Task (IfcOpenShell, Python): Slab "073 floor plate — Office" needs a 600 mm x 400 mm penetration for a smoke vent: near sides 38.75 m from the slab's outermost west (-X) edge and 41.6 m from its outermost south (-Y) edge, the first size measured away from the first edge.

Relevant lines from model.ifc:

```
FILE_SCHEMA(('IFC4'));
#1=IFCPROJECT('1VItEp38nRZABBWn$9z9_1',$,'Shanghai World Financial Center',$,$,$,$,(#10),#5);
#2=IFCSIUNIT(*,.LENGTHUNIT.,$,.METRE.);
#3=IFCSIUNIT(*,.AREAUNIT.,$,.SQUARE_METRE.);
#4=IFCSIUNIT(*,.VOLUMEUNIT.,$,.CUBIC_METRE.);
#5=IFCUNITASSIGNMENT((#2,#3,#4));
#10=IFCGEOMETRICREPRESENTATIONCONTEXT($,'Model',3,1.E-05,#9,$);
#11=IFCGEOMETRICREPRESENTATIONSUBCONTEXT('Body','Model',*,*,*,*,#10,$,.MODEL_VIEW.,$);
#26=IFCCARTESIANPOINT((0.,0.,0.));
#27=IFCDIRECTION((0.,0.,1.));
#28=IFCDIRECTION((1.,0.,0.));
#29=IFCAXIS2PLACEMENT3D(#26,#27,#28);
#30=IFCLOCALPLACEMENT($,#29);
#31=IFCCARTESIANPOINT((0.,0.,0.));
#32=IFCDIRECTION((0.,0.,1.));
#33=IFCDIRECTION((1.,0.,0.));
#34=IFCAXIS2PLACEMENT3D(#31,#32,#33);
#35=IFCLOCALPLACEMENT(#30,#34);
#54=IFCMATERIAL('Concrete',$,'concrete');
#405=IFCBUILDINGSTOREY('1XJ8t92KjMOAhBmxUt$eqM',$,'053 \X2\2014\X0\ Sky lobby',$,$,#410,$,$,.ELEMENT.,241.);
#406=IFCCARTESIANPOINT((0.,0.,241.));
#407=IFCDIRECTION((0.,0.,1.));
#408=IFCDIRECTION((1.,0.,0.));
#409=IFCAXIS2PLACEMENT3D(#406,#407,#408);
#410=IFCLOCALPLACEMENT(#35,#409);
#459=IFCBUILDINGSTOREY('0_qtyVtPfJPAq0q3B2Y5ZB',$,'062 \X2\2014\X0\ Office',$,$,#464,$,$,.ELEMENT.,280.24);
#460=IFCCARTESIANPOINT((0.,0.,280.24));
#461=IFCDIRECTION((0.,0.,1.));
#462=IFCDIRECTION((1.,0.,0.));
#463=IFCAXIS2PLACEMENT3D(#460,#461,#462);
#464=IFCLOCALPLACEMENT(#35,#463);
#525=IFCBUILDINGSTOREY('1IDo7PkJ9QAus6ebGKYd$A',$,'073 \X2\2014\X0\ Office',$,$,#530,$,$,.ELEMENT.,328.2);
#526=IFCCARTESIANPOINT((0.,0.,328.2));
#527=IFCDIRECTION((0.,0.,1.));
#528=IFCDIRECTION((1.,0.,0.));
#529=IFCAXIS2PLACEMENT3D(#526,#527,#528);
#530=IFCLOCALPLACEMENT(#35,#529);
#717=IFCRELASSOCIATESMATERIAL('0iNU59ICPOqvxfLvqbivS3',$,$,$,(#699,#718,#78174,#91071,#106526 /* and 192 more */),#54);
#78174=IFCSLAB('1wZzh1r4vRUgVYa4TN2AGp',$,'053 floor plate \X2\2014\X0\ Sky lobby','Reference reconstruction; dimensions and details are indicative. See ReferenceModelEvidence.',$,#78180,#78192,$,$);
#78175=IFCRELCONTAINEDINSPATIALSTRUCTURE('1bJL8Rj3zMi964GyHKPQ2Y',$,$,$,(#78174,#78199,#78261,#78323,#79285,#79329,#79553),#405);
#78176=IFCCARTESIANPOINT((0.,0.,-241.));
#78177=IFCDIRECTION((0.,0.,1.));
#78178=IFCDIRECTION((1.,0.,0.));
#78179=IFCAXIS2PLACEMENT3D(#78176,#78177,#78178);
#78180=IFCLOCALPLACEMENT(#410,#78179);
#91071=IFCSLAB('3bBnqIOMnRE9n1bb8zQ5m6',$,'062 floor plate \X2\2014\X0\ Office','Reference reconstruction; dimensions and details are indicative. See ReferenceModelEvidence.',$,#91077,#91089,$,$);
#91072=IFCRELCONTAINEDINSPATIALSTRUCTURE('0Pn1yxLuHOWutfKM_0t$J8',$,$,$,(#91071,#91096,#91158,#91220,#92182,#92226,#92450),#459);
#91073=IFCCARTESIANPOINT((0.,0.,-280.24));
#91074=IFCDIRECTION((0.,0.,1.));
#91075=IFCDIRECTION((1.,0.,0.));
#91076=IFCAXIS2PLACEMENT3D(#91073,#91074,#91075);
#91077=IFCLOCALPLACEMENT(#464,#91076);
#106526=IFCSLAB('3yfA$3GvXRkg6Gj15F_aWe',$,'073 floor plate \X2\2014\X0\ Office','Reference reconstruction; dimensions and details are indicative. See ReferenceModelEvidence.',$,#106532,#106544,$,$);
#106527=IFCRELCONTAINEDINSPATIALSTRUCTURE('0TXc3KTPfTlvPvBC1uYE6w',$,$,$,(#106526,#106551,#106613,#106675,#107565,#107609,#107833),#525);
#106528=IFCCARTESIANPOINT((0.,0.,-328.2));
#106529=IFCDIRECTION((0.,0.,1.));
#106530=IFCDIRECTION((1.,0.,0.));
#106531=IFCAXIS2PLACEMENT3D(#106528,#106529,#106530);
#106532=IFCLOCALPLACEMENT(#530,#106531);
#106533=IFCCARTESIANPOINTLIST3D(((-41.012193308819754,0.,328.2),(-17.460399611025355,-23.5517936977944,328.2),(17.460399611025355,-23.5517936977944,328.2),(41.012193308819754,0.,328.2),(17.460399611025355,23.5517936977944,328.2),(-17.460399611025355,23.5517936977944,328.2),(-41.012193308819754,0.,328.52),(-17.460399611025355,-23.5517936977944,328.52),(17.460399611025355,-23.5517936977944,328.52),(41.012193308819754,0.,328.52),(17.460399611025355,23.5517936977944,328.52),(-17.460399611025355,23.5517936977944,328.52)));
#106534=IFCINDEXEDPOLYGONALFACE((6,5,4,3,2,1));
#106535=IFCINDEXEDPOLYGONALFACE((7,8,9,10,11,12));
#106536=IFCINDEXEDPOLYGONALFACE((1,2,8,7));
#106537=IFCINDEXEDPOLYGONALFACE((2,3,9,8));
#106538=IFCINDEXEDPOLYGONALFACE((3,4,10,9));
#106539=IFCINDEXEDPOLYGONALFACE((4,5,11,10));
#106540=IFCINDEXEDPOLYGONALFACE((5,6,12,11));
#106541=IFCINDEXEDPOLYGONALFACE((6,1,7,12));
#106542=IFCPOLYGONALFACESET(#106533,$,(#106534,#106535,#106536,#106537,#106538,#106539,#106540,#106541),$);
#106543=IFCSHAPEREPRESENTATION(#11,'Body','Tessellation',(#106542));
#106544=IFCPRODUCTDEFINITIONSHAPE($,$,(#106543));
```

```python
import numpy as np
import ifcopenshell
import ifcopenshell.api.feature
import ifcopenshell.api.geometry
import ifcopenshell.api.root
import ifcopenshell.geom
import ifcopenshell.util.placement
import ifcopenshell.util.representation
import ifcopenshell.util.shape
import ifcopenshell.util.unit

model = ifcopenshell.open("model.ifc")
unit_scale = ifcopenshell.util.unit.calculate_unit_scale(model)
settings = ifcopenshell.geom.settings()


def volume(element):
    """Net volume in cubic metres, openings subtracted."""
    shape = ifcopenshell.geom.create_shape(settings, element)
    return ifcopenshell.util.shape.get_volume(shape.geometry)


slab = model.by_guid("3yfA$3GvXRkg6Gj15F_aWe")
before = volume(slab)

# Extent in the slab's own axes, in metres. The edges named are its -X and -Y sides.
slab_shape = ifcopenshell.geom.create_shape(settings, slab)
vertices = ifcopenshell.util.shape.get_vertices(slab_shape.geometry)
x_min, y_min, bottom = vertices.min(axis=0)
top = vertices[:, 2].max()

opening = ifcopenshell.api.root.create_entity(model, ifc_class="IfcOpeningElement", name="Smoke vent opening", predefined_type="OPENING")
context = ifcopenshell.util.representation.get_context(model, "Model", "Body", "MODEL_VIEW")
width, depth = 0.6, 0.4
outline = [(0.0, 0.0), (width, 0.0), (width, depth), (0.0, depth), (0.0, 0.0)]
# Overshoot both faces by 50 mm so the cut is clean.
shape = ifcopenshell.api.geometry.add_slab_representation(
    model, context=context, depth=top - bottom + 0.1, polyline=outline
)
ifcopenshell.api.geometry.assign_representation(model, product=opening, representation=shape)

matrix = ifcopenshell.util.placement.get_local_placement(slab.ObjectPlacement)
matrix[:, 3] = matrix @ np.append(np.array([x_min + 38.75, y_min + 41.6, bottom - 0.05]) / unit_scale, 1.0)
ifcopenshell.api.geometry.edit_object_placement(model, product=opening, matrix=matrix, is_si=False)
ifcopenshell.api.feature.add_feature(model, feature=opening, element=slab)

after = volume(slab)

print(f"slab volume {before:.3f} -> {after:.3f} m3")

model.write("model_rev.ifc")
```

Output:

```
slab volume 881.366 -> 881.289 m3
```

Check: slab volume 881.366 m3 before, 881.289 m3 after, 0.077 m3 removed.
